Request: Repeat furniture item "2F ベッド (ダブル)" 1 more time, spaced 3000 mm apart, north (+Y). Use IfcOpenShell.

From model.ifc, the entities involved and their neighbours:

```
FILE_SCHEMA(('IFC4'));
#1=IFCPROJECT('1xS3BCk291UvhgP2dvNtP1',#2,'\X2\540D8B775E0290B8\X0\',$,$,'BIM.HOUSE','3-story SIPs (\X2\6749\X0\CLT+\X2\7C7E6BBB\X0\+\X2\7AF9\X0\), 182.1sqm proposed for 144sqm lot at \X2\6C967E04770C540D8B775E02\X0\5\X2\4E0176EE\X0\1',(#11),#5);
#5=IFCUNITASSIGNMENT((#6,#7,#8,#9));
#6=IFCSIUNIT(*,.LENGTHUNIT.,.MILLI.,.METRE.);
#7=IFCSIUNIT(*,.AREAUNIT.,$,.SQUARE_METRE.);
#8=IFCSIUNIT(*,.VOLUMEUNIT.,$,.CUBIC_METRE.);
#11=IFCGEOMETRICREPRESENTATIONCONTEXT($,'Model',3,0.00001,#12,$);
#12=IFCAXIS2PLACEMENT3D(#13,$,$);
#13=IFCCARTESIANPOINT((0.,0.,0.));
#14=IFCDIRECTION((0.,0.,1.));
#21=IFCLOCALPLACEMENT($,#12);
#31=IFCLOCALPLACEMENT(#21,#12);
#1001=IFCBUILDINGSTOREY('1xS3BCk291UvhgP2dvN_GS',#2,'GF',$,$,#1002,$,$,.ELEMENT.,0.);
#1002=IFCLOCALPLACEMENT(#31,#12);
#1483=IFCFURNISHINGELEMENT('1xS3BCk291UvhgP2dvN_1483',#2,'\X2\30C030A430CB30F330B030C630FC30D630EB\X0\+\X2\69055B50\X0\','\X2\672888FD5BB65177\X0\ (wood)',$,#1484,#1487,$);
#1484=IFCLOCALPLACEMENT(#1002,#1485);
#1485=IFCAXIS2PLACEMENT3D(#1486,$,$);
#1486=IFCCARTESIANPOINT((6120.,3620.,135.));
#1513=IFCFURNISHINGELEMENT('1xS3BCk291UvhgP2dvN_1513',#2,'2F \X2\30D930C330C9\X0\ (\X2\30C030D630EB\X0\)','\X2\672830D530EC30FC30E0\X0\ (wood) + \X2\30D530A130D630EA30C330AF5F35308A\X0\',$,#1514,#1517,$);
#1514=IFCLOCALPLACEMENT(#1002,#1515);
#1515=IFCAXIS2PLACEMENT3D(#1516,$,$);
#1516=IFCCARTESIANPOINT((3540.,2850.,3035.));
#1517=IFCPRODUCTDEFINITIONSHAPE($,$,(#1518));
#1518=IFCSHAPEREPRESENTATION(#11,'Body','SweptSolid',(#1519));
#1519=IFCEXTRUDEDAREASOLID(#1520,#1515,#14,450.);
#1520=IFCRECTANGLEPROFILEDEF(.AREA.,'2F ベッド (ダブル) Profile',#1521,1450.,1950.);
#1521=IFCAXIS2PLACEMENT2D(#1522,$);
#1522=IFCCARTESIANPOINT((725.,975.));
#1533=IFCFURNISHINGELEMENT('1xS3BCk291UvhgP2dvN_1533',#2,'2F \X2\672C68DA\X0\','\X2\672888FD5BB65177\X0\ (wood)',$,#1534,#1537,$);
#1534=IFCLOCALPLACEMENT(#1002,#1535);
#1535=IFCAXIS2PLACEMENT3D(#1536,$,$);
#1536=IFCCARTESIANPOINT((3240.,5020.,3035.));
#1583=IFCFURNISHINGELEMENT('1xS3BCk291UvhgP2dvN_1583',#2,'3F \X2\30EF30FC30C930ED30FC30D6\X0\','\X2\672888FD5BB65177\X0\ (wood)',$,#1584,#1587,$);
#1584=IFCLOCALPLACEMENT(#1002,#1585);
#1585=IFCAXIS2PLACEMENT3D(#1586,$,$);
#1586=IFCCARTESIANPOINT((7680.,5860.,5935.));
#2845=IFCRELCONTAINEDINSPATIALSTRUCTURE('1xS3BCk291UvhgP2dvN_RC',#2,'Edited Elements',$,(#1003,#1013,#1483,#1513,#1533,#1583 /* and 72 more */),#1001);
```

```python
import numpy as np
import ifcopenshell
import ifcopenshell.api.geometry
import ifcopenshell.api.root
import ifcopenshell.util.element
import ifcopenshell.util.placement
import ifcopenshell.util.unit

model = ifcopenshell.open("model.ifc")
unit_scale = ifcopenshell.util.unit.calculate_unit_scale(model)


def reuse_history(source, copy):
    """copy_class also copies each property set's owner history, people and application; keep the originals."""
    for rel in copy.IsDefinedBy:
        if rel.is_a("IfcRelDefinesByProperties") and (history := rel.RelatingPropertyDefinition.OwnerHistory):
            rel.RelatingPropertyDefinition.OwnerHistory = source.OwnerHistory
            ifcopenshell.util.element.remove_deep2(model, history)


source = model.by_guid("1xS3BCk291UvhgP2dvN_1513")
base = ifcopenshell.util.placement.get_local_placement(source.ObjectPlacement)
step = np.array([0.0, 1.0, 0.0]) * 3 / unit_scale

for i in range(1, 2):
    copy = ifcopenshell.api.root.copy_class(model, product=source)
    copy.Representation = ifcopenshell.util.element.copy_deep(
        model, source.Representation, exclude=["IfcGeometricRepresentationContext", "IfcRepresentationMap"]
    )
    reuse_history(source, copy)
    matrix = base.copy()
    matrix[:3, 3] += i * step
    print("added at", matrix[:3, 3].round(3) + 0.0)
    ifcopenshell.api.geometry.edit_object_placement(model, product=copy, matrix=matrix, is_si=False)

model.write("model_edited.ifc")
```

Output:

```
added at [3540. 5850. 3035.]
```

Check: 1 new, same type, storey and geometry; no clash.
